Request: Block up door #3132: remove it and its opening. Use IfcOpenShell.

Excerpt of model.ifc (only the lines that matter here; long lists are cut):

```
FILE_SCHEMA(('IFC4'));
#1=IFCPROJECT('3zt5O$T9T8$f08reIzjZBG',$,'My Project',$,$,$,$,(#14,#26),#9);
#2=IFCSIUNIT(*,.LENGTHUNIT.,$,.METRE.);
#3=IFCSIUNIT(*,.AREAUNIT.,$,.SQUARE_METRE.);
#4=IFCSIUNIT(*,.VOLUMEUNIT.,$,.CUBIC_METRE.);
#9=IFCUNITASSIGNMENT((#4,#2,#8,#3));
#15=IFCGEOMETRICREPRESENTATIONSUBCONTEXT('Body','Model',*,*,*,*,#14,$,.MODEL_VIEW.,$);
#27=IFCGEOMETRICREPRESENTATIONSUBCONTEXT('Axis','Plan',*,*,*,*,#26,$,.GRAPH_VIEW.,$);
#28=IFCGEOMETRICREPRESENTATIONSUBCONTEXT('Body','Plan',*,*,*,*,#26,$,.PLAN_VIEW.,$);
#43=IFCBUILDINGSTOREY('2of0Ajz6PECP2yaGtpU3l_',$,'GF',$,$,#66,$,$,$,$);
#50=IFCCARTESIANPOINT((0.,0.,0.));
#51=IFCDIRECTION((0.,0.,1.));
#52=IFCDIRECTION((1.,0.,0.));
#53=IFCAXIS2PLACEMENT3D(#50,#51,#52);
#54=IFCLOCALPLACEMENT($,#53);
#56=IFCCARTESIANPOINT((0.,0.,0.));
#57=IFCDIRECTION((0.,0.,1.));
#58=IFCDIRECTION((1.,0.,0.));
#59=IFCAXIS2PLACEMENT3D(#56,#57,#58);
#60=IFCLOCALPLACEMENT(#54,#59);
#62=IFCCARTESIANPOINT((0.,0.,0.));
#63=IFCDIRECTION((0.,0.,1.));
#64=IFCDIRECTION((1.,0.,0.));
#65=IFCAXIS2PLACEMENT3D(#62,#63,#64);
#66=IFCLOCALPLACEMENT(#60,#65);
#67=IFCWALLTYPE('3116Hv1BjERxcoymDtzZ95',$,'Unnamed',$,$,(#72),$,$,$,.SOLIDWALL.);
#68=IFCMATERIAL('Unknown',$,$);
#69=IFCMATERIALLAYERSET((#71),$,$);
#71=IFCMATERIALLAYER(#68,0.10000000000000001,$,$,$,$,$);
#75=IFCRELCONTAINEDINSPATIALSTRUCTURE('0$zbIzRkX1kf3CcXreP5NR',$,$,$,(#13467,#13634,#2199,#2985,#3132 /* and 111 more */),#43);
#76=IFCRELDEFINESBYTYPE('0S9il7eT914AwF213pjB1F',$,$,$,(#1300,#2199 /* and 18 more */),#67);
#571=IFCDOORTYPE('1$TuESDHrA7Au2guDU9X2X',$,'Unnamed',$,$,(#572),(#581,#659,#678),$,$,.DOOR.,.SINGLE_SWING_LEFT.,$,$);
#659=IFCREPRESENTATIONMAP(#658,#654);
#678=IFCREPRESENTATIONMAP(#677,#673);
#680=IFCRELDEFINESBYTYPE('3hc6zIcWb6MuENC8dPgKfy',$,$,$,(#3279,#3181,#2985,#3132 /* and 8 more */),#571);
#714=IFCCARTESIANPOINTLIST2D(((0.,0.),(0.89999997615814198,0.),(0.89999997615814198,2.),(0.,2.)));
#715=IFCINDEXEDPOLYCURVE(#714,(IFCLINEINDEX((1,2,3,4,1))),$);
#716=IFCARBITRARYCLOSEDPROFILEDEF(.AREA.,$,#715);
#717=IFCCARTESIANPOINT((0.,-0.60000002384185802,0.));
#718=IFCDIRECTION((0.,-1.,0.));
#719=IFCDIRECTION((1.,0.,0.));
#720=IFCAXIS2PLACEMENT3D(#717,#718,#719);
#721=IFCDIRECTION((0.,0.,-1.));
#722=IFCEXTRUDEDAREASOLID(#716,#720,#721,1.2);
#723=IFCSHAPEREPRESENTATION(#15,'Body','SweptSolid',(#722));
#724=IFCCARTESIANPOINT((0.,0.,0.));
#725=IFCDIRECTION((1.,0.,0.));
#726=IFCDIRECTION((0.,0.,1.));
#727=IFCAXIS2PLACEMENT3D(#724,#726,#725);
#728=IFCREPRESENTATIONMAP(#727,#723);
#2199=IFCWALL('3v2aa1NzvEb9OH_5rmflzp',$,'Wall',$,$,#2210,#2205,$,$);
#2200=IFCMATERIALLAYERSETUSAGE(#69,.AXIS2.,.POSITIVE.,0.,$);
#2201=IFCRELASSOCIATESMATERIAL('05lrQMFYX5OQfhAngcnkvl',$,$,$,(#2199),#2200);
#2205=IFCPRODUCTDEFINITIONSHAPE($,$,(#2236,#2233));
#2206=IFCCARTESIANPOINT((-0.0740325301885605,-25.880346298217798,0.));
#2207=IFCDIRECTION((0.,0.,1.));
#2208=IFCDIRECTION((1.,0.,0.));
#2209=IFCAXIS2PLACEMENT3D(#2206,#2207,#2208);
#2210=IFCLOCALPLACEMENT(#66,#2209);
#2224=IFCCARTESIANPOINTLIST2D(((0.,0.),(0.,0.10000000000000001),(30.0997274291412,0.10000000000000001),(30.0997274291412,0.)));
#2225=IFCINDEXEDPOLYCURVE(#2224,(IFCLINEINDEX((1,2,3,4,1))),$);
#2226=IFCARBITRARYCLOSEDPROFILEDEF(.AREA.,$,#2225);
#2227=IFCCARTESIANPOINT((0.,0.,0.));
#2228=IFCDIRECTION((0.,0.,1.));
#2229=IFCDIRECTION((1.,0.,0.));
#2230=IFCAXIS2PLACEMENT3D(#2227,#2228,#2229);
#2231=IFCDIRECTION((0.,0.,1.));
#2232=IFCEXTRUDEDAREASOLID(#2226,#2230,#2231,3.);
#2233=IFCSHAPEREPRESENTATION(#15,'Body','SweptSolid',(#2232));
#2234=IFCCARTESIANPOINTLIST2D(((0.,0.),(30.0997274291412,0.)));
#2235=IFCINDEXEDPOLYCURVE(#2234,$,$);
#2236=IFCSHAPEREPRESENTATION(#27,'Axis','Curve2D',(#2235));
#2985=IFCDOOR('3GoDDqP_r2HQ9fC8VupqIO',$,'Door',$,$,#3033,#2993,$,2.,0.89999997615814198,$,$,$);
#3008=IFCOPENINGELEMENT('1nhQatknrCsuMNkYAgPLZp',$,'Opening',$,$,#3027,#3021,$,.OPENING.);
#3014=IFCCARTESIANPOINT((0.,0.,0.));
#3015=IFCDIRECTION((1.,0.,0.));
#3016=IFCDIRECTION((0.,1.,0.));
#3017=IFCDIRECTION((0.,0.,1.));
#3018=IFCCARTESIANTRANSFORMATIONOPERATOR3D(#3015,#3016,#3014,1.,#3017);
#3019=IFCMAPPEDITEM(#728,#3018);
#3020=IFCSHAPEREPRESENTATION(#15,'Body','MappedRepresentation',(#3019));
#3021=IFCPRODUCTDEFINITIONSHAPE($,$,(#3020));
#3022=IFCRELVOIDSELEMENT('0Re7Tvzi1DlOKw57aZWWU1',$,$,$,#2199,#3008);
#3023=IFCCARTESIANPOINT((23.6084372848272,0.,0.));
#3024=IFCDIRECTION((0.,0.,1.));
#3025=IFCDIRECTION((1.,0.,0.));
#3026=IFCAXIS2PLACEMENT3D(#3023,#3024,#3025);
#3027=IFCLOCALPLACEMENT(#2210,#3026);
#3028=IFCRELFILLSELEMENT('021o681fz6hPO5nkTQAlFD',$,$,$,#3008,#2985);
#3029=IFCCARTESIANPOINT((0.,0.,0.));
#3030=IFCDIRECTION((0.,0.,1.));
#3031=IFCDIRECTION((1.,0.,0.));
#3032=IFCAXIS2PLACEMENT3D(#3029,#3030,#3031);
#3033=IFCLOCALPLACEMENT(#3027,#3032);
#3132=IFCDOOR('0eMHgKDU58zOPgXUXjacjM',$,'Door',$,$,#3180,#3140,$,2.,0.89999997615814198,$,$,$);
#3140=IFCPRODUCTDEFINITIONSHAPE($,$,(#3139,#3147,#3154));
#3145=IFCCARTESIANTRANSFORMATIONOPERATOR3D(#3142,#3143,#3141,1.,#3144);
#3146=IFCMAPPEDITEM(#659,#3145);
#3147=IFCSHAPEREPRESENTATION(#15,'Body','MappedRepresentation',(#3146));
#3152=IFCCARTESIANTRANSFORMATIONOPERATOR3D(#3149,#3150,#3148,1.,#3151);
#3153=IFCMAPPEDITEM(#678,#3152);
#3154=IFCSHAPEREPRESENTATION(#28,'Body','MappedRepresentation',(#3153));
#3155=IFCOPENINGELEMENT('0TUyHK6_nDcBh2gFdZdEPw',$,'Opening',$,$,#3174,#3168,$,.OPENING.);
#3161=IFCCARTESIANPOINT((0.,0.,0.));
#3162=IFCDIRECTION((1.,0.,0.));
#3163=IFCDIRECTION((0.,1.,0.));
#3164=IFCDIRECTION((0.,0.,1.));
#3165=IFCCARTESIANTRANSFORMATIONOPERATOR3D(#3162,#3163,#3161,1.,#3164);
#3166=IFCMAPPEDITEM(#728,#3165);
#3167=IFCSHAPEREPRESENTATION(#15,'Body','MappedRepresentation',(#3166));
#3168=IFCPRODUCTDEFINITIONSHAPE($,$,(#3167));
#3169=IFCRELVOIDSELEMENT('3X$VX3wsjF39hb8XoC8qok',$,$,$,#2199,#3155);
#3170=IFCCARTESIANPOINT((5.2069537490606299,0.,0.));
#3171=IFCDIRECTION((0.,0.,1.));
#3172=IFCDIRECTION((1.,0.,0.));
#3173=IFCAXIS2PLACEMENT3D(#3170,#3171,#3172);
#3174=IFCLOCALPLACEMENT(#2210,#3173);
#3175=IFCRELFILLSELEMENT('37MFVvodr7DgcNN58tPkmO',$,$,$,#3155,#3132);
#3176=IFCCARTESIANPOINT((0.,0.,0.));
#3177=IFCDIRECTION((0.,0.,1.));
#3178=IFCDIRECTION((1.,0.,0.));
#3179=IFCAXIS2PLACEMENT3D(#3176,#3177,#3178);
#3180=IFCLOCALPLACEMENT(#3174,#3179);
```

```python
import ifcopenshell
import ifcopenshell.api.feature
import ifcopenshell.api.root
import ifcopenshell.geom
import ifcopenshell.util.shape

model = ifcopenshell.open("model.ifc")
settings = ifcopenshell.geom.settings()


def volume(element):
    """Net volume in cubic metres, openings subtracted."""
    shape = ifcopenshell.geom.create_shape(settings, element)
    return ifcopenshell.util.shape.get_volume(shape.geometry)


door = model.by_id(3132)
opening = door.FillsVoids[0].RelatingOpeningElement
wall = opening.VoidsElements[0].RelatingBuildingElement
before = volume(wall)

ifcopenshell.api.root.remove_product(model, product=door)
ifcopenshell.api.feature.remove_feature(model, feature=opening)

after = volume(wall)

print(f"wall volume {before:.3f} -> {after:.3f} m3")

model.write("model_v2.ifc")
```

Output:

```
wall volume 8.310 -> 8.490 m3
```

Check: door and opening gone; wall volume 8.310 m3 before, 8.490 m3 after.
